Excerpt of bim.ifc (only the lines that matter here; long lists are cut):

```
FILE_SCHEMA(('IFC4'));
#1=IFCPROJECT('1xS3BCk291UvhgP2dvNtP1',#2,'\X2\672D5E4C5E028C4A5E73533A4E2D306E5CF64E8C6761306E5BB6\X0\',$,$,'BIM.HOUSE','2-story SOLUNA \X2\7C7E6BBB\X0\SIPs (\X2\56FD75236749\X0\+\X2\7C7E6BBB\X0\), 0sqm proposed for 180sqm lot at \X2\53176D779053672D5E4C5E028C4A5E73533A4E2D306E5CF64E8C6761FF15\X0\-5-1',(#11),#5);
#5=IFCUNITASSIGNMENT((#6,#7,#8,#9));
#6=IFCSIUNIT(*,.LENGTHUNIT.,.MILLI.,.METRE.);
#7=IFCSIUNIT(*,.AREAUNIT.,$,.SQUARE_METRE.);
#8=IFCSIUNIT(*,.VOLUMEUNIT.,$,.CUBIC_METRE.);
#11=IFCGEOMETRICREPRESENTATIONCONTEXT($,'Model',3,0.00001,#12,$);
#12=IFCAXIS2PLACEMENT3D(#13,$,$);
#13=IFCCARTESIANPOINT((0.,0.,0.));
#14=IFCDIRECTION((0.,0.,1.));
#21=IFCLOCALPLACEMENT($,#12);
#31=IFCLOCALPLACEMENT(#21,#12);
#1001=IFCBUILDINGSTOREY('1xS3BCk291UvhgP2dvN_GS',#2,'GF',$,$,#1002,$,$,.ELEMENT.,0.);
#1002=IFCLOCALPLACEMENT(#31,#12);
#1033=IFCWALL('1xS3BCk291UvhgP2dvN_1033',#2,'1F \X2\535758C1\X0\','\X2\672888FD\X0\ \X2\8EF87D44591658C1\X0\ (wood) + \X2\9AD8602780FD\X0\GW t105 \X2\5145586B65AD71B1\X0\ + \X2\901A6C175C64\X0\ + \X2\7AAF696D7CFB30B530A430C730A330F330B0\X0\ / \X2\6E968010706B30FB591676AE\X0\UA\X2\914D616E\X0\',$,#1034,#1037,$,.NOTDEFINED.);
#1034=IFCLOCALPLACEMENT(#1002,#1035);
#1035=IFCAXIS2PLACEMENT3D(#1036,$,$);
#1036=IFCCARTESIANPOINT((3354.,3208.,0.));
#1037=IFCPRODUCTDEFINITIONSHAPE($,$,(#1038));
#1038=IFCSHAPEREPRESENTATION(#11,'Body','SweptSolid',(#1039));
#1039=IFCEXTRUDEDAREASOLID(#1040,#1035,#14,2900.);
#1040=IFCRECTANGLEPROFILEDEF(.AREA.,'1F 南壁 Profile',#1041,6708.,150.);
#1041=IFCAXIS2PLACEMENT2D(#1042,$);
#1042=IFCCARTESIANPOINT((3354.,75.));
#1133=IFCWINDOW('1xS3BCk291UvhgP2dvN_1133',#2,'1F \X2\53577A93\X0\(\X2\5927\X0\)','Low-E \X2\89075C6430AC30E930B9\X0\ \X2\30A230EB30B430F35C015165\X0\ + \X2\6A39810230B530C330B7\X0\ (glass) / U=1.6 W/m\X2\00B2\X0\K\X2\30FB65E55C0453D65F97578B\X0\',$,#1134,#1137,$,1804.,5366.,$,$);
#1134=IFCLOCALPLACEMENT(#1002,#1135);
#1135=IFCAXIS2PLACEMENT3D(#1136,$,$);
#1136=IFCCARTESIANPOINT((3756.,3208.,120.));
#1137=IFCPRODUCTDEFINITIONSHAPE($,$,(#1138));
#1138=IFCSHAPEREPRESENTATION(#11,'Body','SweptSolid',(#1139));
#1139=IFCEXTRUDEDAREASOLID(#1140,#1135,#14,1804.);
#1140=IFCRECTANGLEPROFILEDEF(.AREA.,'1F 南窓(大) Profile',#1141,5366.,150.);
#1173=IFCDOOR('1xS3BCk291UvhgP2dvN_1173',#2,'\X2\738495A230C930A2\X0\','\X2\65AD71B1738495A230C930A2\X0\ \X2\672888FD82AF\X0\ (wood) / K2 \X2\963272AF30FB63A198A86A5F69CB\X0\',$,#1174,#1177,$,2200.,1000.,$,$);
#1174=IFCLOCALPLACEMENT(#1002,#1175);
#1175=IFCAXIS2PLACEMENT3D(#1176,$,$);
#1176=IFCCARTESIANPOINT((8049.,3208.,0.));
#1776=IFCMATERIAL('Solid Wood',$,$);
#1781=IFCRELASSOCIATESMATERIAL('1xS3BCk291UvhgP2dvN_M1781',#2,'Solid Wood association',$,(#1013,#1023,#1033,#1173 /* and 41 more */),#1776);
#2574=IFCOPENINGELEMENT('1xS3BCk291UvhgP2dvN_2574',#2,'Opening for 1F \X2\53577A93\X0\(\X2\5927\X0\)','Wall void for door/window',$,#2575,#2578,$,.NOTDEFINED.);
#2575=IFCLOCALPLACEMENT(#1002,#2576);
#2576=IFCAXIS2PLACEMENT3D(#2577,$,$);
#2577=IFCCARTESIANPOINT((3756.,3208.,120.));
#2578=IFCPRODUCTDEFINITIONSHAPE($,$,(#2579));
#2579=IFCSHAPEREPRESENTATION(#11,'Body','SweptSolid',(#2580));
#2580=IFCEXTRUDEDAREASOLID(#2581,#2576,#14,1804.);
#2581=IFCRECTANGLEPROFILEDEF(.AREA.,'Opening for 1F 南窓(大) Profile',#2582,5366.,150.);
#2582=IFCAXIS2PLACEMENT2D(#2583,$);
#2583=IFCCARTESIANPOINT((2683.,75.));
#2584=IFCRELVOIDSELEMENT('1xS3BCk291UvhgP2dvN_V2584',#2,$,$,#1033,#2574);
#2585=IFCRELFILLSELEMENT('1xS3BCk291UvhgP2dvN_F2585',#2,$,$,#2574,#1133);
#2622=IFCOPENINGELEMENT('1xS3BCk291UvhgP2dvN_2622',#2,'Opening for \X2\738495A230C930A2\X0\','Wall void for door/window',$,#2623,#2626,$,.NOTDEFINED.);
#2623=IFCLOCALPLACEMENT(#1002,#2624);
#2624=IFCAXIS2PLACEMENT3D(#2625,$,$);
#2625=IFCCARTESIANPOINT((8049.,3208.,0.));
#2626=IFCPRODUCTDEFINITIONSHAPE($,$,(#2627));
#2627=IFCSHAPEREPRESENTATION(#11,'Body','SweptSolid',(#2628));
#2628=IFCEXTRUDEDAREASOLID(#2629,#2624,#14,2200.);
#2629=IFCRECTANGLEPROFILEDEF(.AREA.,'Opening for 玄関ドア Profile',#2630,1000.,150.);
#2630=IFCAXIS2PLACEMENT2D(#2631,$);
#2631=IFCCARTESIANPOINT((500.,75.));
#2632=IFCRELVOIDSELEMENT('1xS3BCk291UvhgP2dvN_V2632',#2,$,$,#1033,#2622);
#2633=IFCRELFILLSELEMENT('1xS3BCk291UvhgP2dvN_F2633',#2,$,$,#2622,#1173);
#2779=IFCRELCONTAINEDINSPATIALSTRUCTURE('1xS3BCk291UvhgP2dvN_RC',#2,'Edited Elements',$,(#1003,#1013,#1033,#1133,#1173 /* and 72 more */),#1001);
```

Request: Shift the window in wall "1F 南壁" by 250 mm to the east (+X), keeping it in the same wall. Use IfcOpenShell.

```python
import ifcopenshell
import ifcopenshell.api.geometry
import ifcopenshell.util.placement

model = ifcopenshell.open("bim.ifc")

window = model.by_id(1133)
opening = window.FillsVoids[0].RelatingOpeningElement
wall = opening.VoidsElements[0].RelatingBuildingElement

wall_matrix = ifcopenshell.util.placement.get_local_placement(wall.ObjectPlacement)
shift = wall_matrix[:3, 0] * 250.0
before = ifcopenshell.util.placement.get_local_placement(window.ObjectPlacement)[:3, 3].copy()

# The window is not placed relative to its opening, so move both.
for product in (opening, window):
    matrix = ifcopenshell.util.placement.get_local_placement(product.ObjectPlacement)
    matrix[:3, 3] += shift
    ifcopenshell.api.geometry.edit_object_placement(model, product=product, matrix=matrix, is_si=False)

after = ifcopenshell.util.placement.get_local_placement(window.ObjectPlacement)[:3, 3]
print("window moved by", (after - before).round(3) + 0.0)

model.write("bim_v2.ifc")
```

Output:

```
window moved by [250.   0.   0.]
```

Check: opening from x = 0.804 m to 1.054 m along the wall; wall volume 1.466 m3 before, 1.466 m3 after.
